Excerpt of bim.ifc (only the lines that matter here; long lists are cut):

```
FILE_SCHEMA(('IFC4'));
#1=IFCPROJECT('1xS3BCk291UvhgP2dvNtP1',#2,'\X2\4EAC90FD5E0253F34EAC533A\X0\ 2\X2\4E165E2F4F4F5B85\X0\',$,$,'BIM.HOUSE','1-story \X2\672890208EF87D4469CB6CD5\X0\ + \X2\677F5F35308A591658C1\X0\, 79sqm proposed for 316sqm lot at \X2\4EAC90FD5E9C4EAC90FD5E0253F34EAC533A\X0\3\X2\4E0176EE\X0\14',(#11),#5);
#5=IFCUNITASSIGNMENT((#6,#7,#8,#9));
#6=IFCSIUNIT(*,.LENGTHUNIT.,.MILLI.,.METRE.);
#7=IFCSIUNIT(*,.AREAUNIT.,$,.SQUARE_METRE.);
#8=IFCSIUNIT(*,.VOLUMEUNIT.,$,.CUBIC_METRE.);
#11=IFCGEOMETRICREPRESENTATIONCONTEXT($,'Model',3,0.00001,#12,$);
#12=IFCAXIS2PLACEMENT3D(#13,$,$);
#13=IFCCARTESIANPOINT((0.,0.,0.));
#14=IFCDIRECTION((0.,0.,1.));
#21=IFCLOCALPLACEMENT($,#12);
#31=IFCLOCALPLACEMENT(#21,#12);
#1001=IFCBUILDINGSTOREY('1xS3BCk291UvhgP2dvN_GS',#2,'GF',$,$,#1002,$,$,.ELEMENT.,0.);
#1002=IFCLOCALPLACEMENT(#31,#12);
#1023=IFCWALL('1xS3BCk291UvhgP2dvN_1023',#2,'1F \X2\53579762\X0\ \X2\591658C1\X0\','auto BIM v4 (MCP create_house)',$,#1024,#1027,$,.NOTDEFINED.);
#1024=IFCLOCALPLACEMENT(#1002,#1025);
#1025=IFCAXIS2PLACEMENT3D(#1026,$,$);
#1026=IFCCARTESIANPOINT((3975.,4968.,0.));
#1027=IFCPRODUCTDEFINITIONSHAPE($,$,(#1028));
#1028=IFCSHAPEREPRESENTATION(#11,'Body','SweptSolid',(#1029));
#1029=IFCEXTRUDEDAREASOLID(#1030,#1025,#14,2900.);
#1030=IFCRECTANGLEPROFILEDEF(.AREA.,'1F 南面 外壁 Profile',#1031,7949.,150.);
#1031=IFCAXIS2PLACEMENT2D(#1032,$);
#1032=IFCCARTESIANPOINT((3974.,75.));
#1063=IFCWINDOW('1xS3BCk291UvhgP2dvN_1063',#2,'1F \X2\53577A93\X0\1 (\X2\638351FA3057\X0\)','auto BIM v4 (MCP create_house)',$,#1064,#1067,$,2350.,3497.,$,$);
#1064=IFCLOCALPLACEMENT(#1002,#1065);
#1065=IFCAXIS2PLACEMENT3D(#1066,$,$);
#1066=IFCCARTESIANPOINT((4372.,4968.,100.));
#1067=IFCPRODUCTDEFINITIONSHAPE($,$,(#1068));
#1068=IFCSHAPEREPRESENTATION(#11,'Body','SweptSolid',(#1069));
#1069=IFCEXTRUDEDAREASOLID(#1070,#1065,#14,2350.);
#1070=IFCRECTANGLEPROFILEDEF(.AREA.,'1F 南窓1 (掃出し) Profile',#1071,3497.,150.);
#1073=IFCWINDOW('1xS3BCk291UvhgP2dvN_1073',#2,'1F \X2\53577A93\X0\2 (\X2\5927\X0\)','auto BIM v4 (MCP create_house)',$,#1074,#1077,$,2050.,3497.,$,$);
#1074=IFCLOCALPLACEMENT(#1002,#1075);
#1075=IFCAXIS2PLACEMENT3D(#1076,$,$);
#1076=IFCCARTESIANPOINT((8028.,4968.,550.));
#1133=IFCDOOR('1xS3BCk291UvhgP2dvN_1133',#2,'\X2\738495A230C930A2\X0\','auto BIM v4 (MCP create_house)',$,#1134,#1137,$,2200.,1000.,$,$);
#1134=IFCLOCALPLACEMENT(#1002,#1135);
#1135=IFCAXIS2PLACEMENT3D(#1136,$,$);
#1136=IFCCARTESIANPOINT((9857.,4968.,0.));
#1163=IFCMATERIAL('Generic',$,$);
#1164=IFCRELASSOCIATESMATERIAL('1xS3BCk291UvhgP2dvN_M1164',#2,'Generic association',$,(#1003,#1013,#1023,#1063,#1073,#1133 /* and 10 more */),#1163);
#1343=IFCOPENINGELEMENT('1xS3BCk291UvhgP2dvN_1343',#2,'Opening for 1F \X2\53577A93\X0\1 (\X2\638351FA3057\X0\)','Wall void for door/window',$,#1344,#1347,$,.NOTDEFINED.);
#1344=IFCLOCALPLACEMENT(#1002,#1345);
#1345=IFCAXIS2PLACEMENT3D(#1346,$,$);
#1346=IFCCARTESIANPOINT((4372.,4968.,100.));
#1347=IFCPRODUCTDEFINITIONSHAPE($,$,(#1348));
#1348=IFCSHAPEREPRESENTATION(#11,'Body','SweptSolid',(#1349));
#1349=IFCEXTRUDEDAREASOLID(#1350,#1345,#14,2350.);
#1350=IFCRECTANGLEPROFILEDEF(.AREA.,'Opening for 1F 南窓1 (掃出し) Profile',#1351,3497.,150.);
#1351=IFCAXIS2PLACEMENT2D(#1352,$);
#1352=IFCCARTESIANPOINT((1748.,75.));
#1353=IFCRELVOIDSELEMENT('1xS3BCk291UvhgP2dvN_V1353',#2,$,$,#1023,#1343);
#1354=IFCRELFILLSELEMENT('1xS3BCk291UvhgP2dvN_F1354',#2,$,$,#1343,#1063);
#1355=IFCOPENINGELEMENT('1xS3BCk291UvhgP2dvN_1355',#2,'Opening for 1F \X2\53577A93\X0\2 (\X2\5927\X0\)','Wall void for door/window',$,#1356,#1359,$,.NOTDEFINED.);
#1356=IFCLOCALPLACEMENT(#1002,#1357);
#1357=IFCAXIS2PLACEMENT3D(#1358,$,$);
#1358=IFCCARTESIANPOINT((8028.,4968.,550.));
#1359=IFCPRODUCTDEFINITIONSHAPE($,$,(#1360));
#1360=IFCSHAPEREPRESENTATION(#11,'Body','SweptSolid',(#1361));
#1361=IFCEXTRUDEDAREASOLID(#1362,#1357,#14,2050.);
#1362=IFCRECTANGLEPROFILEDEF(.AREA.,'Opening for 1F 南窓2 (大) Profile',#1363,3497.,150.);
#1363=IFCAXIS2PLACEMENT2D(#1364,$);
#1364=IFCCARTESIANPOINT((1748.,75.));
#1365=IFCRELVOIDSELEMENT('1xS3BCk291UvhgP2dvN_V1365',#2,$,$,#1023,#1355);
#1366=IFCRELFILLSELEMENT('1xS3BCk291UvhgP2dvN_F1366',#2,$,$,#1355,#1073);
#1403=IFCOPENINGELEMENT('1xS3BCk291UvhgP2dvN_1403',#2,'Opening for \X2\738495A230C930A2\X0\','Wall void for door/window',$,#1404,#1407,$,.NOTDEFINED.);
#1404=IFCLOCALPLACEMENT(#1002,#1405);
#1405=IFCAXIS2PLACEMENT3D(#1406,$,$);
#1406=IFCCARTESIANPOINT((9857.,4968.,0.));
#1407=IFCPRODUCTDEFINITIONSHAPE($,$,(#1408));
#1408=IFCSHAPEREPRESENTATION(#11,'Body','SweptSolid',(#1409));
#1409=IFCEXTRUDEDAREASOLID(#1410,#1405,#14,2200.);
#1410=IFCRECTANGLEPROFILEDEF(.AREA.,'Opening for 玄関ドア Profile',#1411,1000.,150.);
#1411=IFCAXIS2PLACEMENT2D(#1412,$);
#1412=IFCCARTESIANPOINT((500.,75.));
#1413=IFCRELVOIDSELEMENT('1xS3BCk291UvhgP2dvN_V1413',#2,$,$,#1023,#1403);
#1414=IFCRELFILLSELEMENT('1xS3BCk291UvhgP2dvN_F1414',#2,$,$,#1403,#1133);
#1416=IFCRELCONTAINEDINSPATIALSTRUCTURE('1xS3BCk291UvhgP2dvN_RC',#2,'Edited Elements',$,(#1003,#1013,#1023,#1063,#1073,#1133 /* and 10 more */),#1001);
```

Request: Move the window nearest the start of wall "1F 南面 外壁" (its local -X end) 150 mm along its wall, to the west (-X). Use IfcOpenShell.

```python
import ifcopenshell
import ifcopenshell.api.geometry
import ifcopenshell.util.placement
import ifcopenshell.util.unit

model = ifcopenshell.open("bim.ifc")
unit_scale = ifcopenshell.util.unit.calculate_unit_scale(model)

window = model.by_guid("1xS3BCk291UvhgP2dvN_1063")
opening = window.FillsVoids[0].RelatingOpeningElement
wall = opening.VoidsElements[0].RelatingBuildingElement

wall_matrix = ifcopenshell.util.placement.get_local_placement(wall.ObjectPlacement)
shift = wall_matrix[:3, 0] * -0.15 / unit_scale
before = ifcopenshell.util.placement.get_local_placement(window.ObjectPlacement)[:3, 3].copy()

# The window is not placed relative to its opening, so move both.
for product in (opening, window):
    matrix = ifcopenshell.util.placement.get_local_placement(product.ObjectPlacement)
    matrix[:3, 3] += shift
    ifcopenshell.api.geometry.edit_object_placement(model, product=product, matrix=matrix, is_si=False)

after = ifcopenshell.util.placement.get_local_placement(window.ObjectPlacement)[:3, 3]
print("window moved by", (after - before).round(3) + 0.0)

model.write("bim_edited.ifc")
```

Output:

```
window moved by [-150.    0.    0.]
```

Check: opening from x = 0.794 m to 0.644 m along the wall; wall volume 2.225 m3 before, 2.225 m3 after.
